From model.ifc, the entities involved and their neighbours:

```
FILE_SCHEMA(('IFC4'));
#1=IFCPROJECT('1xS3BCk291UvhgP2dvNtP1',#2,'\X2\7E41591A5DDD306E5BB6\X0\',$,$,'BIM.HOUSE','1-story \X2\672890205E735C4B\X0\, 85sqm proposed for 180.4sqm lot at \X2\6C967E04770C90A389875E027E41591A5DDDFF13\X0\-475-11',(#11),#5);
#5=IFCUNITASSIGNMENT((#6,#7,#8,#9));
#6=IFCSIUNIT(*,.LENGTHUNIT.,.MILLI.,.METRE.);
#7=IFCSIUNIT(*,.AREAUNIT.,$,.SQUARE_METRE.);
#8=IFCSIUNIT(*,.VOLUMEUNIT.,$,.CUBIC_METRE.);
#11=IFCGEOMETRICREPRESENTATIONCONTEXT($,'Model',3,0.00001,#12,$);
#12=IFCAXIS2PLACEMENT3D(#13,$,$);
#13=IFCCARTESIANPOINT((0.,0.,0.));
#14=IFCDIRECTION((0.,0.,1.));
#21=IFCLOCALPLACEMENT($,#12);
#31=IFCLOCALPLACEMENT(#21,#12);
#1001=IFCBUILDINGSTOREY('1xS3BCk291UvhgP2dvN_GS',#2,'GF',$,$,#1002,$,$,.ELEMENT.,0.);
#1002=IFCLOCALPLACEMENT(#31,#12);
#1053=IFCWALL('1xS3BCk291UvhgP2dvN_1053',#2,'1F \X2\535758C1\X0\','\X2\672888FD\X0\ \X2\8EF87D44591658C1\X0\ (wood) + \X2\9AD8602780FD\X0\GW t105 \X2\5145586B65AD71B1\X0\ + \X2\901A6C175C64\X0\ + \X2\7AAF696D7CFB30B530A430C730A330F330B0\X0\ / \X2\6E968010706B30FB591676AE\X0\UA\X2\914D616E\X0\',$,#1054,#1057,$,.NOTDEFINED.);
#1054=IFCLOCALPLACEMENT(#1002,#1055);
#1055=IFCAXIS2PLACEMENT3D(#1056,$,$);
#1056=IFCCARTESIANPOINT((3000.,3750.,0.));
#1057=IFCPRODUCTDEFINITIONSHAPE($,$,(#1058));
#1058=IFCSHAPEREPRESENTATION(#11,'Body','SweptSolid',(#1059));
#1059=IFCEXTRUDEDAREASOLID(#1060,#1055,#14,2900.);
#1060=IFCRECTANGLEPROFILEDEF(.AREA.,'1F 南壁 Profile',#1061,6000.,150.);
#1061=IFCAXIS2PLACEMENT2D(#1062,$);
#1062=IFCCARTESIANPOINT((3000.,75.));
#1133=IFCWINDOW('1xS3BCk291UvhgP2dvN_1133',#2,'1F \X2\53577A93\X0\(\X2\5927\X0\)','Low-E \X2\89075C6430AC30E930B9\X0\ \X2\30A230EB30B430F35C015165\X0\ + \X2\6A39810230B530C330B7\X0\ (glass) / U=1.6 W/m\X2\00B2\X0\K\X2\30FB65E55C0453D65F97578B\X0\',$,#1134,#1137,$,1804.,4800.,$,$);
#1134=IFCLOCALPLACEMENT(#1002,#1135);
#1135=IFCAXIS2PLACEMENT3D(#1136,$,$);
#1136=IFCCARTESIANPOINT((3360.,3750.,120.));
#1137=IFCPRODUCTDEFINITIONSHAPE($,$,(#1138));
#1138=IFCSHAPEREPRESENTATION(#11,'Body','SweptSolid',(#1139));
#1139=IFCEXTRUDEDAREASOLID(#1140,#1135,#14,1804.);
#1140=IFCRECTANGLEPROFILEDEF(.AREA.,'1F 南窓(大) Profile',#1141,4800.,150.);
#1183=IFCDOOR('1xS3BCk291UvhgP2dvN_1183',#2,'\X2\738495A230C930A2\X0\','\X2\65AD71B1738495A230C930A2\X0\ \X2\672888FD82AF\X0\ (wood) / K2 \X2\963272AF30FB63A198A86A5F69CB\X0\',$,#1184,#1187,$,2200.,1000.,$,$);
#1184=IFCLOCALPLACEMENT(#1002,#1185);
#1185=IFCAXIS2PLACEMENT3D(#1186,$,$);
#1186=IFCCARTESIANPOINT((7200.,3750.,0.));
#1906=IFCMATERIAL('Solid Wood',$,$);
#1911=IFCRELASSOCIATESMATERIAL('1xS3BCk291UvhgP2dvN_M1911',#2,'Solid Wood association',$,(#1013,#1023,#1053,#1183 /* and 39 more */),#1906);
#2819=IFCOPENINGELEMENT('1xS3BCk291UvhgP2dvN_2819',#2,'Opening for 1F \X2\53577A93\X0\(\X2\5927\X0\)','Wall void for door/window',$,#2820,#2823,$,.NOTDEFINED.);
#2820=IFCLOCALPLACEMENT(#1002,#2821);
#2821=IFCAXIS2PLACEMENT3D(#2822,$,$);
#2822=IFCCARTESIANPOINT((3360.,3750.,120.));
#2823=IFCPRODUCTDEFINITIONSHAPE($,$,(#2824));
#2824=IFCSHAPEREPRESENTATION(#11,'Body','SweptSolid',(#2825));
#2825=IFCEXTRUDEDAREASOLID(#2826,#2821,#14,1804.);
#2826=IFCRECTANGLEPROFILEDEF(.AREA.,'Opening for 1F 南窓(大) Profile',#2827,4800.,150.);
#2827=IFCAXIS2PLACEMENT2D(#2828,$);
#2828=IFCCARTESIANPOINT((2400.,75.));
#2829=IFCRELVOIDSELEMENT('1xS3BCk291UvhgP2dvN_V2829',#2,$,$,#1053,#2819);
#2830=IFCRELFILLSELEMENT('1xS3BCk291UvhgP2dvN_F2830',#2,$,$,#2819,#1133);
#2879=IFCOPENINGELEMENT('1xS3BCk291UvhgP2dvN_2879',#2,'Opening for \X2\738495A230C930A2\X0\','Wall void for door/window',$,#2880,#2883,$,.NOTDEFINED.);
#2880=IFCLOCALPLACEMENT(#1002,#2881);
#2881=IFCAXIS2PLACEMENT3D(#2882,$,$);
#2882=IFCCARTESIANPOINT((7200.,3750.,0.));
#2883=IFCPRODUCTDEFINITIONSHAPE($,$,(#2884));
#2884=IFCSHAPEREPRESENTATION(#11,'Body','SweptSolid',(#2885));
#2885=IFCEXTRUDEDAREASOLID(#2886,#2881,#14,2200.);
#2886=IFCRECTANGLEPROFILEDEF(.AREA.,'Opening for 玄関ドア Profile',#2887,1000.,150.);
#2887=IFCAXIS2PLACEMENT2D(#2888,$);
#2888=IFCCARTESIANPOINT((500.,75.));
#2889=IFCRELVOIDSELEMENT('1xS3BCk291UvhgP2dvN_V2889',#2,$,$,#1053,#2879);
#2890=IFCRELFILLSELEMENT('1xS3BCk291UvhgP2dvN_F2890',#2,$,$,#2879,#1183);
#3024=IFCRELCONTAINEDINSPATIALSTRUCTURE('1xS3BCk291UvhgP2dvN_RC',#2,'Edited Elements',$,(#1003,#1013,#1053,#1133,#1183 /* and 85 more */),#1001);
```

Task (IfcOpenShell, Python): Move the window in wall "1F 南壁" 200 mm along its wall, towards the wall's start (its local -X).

```python
import ifcopenshell
import ifcopenshell.api.geometry
import ifcopenshell.util.placement

model = ifcopenshell.open("model.ifc")

window = model.by_guid("1xS3BCk291UvhgP2dvN_1133")
opening = window.FillsVoids[0].RelatingOpeningElement
wall = opening.VoidsElements[0].RelatingBuildingElement

wall_matrix = ifcopenshell.util.placement.get_local_placement(wall.ObjectPlacement)
shift = wall_matrix[:3, 0] * -200.0
before = ifcopenshell.util.placement.get_local_placement(window.ObjectPlacement)[:3, 3].copy()

# The window is not placed relative to its opening, so move both.
for product in (opening, window):
    matrix = ifcopenshell.util.placement.get_local_placement(product.ObjectPlacement)
    matrix[:3, 3] += shift
    ifcopenshell.api.geometry.edit_object_placement(model, product=product, matrix=matrix, is_si=False)

after = ifcopenshell.util.placement.get_local_placement(window.ObjectPlacement)[:3, 3]
print("window moved by", (after - before).round(3) + 0.0)

model.write("model_rev.ifc")
```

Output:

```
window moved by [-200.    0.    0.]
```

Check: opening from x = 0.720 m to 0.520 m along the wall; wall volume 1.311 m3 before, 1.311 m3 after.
